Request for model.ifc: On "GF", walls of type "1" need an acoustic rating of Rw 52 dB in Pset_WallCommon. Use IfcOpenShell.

First a look at what the model holds.

```python
import ifcopenshell
import ifcopenshell.util.element

model = ifcopenshell.open("model.ifc")
print(model.schema)
storey = next(s for s in model.by_type("IfcBuildingStorey") if s.Name == "GF")
walls = [e for e in ifcopenshell.util.element.get_decomposition(storey) if e.is_a("IfcWall")]
seen = {}
for e in walls:
    element_type = ifcopenshell.util.element.get_type(e)
    key = (element_type.Name if element_type != e and element_type else None, ifcopenshell.util.element.get_pset(e, "Pset_WallCommon", "AcousticRating"))
    seen[key] = seen.get(key, 0) + 1
for (name, value), count in sorted(seen.items(), key=str):
    print(count, "x", name, "|", value)
```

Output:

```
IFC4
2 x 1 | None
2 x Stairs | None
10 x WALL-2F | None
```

```python
import ifcopenshell
import ifcopenshell.api.pset
import ifcopenshell.util.element

model = ifcopenshell.open("model.ifc")

storey = next(s for s in model.by_type("IfcBuildingStorey") if s.Name == "GF")
walls = [e for e in ifcopenshell.util.element.get_decomposition(storey) if e.is_a("IfcWall")]

count = 0
for e in walls:
    element_type = ifcopenshell.util.element.get_type(e)
    if element_type in (None, e) or element_type.Name != "1":
        continue
    # add_pset returns the element's existing set when there is one.
    pset = ifcopenshell.api.pset.add_pset(model, product=e, name="Pset_WallCommon")
    ifcopenshell.api.pset.edit_pset(model, pset=pset, properties={"AcousticRating": "Rw 52 dB"})
    count += 1

print(count, "walls updated")

model.write("model_edited.ifc")
```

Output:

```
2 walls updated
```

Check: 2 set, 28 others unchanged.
